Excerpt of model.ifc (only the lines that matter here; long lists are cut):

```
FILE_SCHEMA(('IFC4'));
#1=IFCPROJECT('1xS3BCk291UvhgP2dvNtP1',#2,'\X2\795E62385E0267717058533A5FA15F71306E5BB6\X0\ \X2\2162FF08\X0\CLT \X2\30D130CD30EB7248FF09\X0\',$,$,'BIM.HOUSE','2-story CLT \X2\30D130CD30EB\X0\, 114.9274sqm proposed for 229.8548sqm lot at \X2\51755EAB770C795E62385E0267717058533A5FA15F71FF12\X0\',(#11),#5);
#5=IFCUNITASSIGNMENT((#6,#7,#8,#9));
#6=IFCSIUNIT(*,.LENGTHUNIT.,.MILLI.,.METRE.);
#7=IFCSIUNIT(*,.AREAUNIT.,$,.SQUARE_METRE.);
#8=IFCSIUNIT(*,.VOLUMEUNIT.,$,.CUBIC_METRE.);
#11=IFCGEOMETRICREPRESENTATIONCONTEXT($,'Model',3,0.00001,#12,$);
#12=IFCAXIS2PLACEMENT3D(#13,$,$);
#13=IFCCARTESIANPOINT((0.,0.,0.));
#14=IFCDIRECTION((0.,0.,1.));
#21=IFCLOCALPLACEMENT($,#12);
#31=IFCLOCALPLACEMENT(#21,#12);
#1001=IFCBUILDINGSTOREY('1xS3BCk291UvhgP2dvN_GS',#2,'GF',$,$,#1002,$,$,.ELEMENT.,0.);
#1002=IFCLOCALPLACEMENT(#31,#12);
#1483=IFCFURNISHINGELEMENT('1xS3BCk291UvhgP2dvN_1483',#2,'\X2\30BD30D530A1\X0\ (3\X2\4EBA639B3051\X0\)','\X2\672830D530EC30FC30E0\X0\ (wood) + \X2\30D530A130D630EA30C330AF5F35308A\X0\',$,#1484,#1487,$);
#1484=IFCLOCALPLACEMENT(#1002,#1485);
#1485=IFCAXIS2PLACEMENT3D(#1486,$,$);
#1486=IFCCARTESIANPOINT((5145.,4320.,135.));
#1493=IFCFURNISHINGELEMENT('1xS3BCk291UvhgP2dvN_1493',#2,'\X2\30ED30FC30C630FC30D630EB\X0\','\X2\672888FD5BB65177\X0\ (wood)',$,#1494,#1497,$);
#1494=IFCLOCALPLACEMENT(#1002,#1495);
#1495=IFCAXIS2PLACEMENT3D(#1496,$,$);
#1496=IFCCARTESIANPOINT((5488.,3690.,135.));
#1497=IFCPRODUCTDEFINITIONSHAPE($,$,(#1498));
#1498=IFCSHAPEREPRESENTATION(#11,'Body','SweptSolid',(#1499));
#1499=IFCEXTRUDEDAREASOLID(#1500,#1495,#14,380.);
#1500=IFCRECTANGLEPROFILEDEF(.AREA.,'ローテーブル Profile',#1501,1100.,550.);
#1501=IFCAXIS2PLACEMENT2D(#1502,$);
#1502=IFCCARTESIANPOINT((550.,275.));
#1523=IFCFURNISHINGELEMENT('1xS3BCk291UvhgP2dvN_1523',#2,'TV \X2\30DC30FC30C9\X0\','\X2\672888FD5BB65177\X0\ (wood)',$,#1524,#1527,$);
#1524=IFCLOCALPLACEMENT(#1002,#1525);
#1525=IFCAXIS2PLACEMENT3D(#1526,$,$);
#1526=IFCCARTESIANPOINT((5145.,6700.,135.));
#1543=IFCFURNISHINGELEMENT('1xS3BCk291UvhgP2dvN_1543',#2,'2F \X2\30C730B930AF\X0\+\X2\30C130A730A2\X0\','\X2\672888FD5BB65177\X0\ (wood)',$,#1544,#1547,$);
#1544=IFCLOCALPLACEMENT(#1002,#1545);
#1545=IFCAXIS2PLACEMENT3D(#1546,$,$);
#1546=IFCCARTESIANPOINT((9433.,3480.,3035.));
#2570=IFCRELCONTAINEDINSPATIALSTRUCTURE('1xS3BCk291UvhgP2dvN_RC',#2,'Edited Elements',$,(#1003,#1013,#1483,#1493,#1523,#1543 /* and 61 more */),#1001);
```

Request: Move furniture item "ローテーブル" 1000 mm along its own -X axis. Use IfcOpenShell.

```python
import ifcopenshell
import ifcopenshell.api.geometry
import ifcopenshell.util.placement
import ifcopenshell.util.unit

model = ifcopenshell.open("model.ifc")
unit_scale = ifcopenshell.util.unit.calculate_unit_scale(model)

item = model.by_id(1493)
matrix = ifcopenshell.util.placement.get_local_placement(item.ObjectPlacement)
matrix[:3, 3] -= matrix[:3, 0] * 1 / unit_scale
ifcopenshell.api.geometry.edit_object_placement(model, product=item, matrix=matrix, is_si=False)

print(ifcopenshell.util.placement.get_local_placement(item.ObjectPlacement).round(3) + 0.0)

model.write("model_updated.ifc")
```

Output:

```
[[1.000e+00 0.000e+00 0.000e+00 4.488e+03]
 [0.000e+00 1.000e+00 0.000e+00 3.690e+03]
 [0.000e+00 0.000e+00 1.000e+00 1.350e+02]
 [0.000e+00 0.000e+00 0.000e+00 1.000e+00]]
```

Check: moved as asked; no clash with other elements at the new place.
